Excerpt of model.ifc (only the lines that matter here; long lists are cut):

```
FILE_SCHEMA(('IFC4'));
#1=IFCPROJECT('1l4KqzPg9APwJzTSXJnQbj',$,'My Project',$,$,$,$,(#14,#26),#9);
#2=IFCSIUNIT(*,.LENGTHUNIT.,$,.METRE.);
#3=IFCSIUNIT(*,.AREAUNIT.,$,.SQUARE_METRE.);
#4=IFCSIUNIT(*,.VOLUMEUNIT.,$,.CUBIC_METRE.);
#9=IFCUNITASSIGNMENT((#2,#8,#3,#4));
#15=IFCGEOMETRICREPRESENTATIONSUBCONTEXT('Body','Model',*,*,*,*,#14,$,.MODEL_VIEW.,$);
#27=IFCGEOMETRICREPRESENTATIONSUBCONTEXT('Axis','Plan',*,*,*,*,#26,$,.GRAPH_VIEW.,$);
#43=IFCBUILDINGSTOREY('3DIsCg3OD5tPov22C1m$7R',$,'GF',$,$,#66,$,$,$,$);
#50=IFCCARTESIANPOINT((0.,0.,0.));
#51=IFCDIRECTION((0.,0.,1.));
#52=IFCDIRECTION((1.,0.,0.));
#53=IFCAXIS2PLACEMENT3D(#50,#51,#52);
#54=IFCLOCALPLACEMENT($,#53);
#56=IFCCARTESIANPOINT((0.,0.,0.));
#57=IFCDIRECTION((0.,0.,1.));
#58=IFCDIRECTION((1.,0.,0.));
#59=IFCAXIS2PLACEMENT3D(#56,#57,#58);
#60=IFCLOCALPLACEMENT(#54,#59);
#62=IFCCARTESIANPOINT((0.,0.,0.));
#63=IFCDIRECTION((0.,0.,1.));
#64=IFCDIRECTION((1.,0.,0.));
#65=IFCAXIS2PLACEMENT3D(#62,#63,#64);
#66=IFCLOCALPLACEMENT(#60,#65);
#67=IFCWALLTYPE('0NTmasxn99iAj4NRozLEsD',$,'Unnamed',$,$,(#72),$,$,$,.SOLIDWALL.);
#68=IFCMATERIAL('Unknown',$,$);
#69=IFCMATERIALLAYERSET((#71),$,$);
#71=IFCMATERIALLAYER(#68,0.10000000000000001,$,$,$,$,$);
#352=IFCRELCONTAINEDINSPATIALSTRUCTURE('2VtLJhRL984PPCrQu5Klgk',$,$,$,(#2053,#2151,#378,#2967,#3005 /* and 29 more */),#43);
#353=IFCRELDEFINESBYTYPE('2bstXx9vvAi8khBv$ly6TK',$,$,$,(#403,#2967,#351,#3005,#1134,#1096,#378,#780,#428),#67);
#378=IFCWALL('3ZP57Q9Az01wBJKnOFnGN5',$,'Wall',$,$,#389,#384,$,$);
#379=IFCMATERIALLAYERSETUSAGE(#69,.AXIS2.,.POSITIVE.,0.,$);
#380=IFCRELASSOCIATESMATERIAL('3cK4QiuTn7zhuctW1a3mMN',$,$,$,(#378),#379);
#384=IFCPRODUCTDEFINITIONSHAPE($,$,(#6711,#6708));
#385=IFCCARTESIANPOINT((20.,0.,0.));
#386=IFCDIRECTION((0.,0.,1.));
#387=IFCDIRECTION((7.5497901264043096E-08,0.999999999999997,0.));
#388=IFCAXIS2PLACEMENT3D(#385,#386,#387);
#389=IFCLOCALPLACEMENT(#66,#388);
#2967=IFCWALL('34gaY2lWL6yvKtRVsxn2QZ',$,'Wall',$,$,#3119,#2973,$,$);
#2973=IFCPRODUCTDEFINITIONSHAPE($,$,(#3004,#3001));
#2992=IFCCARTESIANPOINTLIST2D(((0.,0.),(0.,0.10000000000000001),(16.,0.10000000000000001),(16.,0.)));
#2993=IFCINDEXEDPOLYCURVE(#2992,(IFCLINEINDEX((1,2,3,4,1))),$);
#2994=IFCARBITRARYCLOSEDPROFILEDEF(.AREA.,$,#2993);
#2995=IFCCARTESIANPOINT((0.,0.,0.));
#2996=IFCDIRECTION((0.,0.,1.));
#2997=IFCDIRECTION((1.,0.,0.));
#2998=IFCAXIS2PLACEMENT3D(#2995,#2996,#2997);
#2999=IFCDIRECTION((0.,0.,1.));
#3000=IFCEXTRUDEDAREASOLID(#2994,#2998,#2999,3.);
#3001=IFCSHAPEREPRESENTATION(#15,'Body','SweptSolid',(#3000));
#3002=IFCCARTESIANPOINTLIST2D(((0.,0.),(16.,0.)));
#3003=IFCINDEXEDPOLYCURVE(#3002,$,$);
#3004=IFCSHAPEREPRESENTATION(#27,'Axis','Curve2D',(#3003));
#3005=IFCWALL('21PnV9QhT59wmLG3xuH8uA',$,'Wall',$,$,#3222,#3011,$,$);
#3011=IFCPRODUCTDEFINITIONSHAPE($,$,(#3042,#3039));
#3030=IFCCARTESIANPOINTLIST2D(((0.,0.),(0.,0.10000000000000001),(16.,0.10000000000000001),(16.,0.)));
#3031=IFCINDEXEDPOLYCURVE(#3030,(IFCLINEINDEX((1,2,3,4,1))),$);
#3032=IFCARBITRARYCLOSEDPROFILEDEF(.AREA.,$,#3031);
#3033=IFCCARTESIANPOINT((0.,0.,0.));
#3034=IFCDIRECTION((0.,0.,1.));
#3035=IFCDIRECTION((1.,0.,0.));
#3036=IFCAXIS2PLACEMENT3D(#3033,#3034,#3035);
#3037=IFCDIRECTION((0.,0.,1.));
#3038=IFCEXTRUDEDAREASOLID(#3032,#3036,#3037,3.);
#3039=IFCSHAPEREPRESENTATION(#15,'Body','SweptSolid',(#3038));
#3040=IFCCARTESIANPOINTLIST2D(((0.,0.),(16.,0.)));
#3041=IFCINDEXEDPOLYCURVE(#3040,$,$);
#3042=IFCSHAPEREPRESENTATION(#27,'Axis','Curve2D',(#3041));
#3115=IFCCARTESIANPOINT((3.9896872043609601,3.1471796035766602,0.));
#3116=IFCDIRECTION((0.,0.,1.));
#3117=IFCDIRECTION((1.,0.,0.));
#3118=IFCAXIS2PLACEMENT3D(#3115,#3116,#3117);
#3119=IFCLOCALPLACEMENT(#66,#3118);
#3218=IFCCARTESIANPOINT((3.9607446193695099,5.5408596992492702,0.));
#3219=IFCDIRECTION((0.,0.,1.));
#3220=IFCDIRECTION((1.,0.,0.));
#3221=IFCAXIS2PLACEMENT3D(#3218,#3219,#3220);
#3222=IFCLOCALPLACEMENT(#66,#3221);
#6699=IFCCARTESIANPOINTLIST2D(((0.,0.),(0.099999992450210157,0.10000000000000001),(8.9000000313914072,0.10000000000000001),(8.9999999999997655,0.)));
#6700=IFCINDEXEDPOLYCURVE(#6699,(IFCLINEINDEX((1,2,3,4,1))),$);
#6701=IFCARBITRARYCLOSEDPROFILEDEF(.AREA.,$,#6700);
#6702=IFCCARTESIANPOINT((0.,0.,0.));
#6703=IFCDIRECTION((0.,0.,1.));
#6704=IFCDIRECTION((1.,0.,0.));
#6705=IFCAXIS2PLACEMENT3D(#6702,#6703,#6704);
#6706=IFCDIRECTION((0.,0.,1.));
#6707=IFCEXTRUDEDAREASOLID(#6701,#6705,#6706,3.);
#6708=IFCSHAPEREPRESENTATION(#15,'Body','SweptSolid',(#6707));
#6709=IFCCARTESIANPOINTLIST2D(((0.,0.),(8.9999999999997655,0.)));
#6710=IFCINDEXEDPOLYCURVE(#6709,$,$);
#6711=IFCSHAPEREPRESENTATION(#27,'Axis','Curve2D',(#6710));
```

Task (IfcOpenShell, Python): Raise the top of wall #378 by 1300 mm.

```python
import ifcopenshell
import ifcopenshell.geom
import ifcopenshell.util.representation
import ifcopenshell.util.shape

model = ifcopenshell.open("model.ifc")
settings = ifcopenshell.geom.settings()


def volume(element):
    """Net volume in cubic metres, openings subtracted."""
    shape = ifcopenshell.geom.create_shape(settings, element)
    return ifcopenshell.util.shape.get_volume(shape.geometry)


wall = model.by_guid("3ZP57Q9Az01wBJKnOFnGN5")
before = volume(wall)

body = ifcopenshell.util.representation.get_representation(wall, "Model", "Body")
solid = body.Items[0]
old_height = solid.Depth
solid.Depth += 1.3
after = volume(wall)

print(f"height {old_height:g} -> {solid.Depth:g}, volume {before:.3f} -> {after:.3f} m3")

model.write("model_v2.ifc")
```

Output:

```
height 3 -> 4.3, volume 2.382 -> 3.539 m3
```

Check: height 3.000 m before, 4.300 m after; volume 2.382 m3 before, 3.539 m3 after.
